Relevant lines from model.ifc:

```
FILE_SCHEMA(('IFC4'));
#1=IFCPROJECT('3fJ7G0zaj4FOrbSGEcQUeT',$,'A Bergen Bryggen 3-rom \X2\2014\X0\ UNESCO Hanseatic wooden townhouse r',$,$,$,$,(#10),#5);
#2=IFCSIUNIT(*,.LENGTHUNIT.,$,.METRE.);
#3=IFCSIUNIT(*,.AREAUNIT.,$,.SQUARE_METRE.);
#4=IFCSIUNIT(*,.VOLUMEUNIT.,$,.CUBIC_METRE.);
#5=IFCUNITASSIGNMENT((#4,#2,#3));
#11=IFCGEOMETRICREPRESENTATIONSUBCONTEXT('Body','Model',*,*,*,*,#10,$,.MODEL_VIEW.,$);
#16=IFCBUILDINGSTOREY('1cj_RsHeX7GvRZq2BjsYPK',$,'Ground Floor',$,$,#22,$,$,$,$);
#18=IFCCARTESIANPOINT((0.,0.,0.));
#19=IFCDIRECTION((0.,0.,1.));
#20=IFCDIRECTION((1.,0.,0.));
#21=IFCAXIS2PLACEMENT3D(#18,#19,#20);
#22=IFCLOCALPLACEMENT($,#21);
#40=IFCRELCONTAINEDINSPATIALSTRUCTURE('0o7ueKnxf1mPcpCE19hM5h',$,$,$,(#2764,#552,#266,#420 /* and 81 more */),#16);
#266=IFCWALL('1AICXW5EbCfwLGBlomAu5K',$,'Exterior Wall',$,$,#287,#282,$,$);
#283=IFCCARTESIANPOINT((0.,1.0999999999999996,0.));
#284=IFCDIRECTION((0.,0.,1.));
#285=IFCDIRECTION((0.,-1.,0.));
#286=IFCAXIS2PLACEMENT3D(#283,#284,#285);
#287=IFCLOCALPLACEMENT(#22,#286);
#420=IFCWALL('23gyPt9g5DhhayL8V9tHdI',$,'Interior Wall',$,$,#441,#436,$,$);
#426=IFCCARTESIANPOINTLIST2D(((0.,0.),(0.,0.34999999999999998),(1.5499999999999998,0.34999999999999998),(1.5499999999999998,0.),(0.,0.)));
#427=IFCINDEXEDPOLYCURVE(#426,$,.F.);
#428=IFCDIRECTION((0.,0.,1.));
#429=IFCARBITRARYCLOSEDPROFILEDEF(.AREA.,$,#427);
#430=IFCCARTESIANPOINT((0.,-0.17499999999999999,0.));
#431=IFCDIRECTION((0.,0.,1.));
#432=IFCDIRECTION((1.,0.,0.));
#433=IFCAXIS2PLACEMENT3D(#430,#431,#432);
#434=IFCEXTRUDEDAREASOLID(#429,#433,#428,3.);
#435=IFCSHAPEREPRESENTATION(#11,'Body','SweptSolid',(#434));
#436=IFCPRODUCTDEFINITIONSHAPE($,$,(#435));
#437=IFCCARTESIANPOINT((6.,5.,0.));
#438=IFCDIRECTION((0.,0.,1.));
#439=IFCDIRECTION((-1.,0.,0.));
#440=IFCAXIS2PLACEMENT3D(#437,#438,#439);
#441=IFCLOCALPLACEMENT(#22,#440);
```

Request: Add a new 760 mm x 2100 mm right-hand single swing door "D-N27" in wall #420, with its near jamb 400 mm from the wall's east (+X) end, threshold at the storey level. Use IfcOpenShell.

```python
import numpy as np
import ifcopenshell
import ifcopenshell.api.feature
import ifcopenshell.api.geometry
import ifcopenshell.api.root
import ifcopenshell.api.spatial
import ifcopenshell.geom
import ifcopenshell.util.element
import ifcopenshell.util.placement
import ifcopenshell.util.representation
import ifcopenshell.util.shape
import ifcopenshell.util.unit

model = ifcopenshell.open("model.ifc")
unit_scale = ifcopenshell.util.unit.calculate_unit_scale(model)
settings = ifcopenshell.geom.settings()


def volume(element):
    """Net volume in cubic metres, openings subtracted."""
    shape = ifcopenshell.geom.create_shape(settings, element)
    return ifcopenshell.util.shape.get_volume(shape.geometry)


wall = model.by_guid("23gyPt9g5DhhayL8V9tHdI")
storey = ifcopenshell.util.element.get_container(wall, ifc_class="IfcBuildingStorey")
context = ifcopenshell.util.representation.get_context(model, "Model", "Body", "MODEL_VIEW")
before = volume(wall)

width, height, from_end, sill = 0.76, 2.1, 0.4, 0.0  # metres

# The wall runs along its own X axis, and the end named is its -X end.
wall_shape = ifcopenshell.geom.create_shape(settings, wall)
x, y, z = ifcopenshell.util.shape.get_vertices(wall_shape.geometry).T
start = x.min() + from_end
face, thickness = float(y.min()), float(y.max() - y.min())
wall_matrix = ifcopenshell.util.placement.get_local_placement(wall.ObjectPlacement)
level = ifcopenshell.util.placement.get_local_placement(storey.ObjectPlacement)[2, 3]


def in_wall(x, y):
    """Placement at x, y metres in the wall's axes, at sill height."""
    matrix = wall_matrix.copy()
    matrix[:, 3] = wall_matrix @ np.array([x / unit_scale, y / unit_scale, 0.0, 1.0])
    matrix[2, 3] = level + sill / unit_scale
    return matrix


# Opening: a box that overshoots both wall faces by 50 mm.
opening = ifcopenshell.api.root.create_entity(model, ifc_class="IfcOpeningElement", predefined_type="OPENING")
box = ifcopenshell.api.geometry.add_wall_representation(
    model, context=context, length=width, height=height, thickness=thickness + 0.1
)
ifcopenshell.api.geometry.assign_representation(model, product=opening, representation=box)
ifcopenshell.api.geometry.edit_object_placement(model, product=opening, matrix=in_wall(start, face - 0.05), is_si=False)
ifcopenshell.api.feature.add_feature(model, feature=opening, element=wall)

door = ifcopenshell.api.root.create_entity(model, ifc_class="IfcDoor", name="D-N27", predefined_type="DOOR")
door.OverallWidth, door.OverallHeight = width / unit_scale, height / unit_scale
door.OperationType = "SINGLE_SWING_RIGHT"
body = ifcopenshell.api.geometry.add_door_representation(
    model,
    context=context,
    overall_width=door.OverallWidth,
    overall_height=door.OverallHeight,
    operation_type="SINGLE_SWING_RIGHT",
    lining_properties={"LiningDepth": thickness / unit_scale, "ThresholdDepth": thickness / unit_scale},
)
ifcopenshell.api.geometry.assign_representation(model, product=door, representation=body)
ifcopenshell.api.spatial.assign_container(model, products=[door], relating_structure=storey)
ifcopenshell.api.feature.add_filling(model, opening=opening, element=door)

# The lining spans the wall, so the door starts at the wall face.
ifcopenshell.api.geometry.edit_object_placement(model, product=door, matrix=in_wall(start, face), is_si=False)

after = volume(wall)

print(f"wall volume {before:.3f} -> {after:.3f} m3")

model.write("model_edited.ifc")
```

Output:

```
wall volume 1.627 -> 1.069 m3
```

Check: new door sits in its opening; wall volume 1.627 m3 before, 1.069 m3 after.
